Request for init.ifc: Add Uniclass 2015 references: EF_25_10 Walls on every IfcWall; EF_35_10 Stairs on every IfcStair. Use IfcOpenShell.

First a look at what the model holds.

```python
import ifcopenshell

model = ifcopenshell.open("init.ifc")
print(model.schema)
print("classifications:", [c.Name for c in model.by_type("IfcClassification")])
for ifc_class in ("IfcDoor", "IfcRoof", "IfcStair", "IfcWall", "IfcWindow"):
    print(ifc_class, len(model.by_type(ifc_class)))
```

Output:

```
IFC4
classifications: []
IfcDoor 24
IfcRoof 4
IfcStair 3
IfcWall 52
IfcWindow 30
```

```python
import ifcopenshell
import ifcopenshell.api.classification

model = ifcopenshell.open("init.ifc")

system = ifcopenshell.api.classification.add_classification(model, classification="Uniclass 2015")

codes = {
    "IfcWall": ("EF_25_10", "Walls"),
    "IfcStair": ("EF_35_10", "Stairs"),
}
for ifc_class, (code, name) in codes.items():
    products = model.by_type(ifc_class)
    ifcopenshell.api.classification.add_reference(
        model, products=products, classification=system, identification=code, name=name
    )
    print(code, len(products))

model.write("init-out.ifc")
```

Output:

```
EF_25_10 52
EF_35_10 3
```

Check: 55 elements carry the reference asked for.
